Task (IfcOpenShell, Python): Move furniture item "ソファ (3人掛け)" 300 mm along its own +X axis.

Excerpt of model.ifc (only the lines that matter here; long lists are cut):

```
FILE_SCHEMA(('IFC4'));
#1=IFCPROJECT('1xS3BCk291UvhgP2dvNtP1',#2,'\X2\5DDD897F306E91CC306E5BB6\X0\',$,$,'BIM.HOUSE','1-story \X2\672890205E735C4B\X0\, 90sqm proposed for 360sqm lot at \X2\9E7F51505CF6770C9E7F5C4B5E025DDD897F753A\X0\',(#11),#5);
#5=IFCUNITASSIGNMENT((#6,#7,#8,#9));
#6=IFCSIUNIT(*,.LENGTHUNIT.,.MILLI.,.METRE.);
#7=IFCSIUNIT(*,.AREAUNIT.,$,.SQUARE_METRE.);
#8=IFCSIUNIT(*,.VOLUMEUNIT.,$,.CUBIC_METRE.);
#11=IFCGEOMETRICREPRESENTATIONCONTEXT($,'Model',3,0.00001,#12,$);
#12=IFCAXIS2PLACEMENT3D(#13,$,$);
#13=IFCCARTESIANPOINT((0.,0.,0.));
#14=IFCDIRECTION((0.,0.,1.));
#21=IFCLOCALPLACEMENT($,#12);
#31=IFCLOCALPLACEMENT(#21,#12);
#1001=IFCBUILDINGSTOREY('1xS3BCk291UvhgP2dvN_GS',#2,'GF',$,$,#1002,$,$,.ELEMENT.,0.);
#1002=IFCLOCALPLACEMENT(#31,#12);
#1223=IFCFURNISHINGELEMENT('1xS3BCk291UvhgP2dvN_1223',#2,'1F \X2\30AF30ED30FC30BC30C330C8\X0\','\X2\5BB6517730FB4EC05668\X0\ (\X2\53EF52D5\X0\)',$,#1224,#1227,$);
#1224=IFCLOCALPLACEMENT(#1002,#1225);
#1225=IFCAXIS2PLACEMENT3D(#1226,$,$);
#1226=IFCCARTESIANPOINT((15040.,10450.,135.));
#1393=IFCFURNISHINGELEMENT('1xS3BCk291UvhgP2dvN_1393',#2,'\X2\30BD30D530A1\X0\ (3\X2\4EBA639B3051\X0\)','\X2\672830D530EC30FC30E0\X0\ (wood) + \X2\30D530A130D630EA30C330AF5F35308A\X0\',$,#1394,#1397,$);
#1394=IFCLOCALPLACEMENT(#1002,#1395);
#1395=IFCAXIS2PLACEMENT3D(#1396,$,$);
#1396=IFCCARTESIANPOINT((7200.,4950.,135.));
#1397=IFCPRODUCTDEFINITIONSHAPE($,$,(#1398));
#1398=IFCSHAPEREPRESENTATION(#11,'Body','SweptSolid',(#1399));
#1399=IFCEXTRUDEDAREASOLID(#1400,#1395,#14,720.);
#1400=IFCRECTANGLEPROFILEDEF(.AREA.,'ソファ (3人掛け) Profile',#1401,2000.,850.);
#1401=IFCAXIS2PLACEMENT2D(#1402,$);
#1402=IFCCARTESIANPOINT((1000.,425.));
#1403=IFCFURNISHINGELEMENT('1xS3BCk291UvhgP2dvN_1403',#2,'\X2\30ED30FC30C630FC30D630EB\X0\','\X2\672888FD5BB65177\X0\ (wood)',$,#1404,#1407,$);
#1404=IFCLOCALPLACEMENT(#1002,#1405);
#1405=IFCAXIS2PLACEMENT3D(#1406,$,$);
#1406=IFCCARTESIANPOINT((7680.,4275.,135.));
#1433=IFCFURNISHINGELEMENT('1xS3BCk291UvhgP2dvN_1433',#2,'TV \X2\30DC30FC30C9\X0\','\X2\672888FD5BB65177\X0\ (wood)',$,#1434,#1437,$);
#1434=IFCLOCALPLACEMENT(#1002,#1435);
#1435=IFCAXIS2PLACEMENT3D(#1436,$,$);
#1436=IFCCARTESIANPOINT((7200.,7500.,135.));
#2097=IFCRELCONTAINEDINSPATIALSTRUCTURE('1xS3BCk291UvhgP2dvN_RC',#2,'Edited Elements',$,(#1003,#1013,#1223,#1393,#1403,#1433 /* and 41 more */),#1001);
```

```python
import ifcopenshell
import ifcopenshell.api.geometry
import ifcopenshell.util.placement
import ifcopenshell.util.unit

model = ifcopenshell.open("model.ifc")
unit_scale = ifcopenshell.util.unit.calculate_unit_scale(model)

item = model.by_guid("1xS3BCk291UvhgP2dvN_1393")
matrix = ifcopenshell.util.placement.get_local_placement(item.ObjectPlacement)
matrix[:3, 3] += matrix[:3, 0] * 0.3 / unit_scale
ifcopenshell.api.geometry.edit_object_placement(model, product=item, matrix=matrix, is_si=False)

print(ifcopenshell.util.placement.get_local_placement(item.ObjectPlacement).round(3) + 0.0)

model.write("model_v2.ifc")
```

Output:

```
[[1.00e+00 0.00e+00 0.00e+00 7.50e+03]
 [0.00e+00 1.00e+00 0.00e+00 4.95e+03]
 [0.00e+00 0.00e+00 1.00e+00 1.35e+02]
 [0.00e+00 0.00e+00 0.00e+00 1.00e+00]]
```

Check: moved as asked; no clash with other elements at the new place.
